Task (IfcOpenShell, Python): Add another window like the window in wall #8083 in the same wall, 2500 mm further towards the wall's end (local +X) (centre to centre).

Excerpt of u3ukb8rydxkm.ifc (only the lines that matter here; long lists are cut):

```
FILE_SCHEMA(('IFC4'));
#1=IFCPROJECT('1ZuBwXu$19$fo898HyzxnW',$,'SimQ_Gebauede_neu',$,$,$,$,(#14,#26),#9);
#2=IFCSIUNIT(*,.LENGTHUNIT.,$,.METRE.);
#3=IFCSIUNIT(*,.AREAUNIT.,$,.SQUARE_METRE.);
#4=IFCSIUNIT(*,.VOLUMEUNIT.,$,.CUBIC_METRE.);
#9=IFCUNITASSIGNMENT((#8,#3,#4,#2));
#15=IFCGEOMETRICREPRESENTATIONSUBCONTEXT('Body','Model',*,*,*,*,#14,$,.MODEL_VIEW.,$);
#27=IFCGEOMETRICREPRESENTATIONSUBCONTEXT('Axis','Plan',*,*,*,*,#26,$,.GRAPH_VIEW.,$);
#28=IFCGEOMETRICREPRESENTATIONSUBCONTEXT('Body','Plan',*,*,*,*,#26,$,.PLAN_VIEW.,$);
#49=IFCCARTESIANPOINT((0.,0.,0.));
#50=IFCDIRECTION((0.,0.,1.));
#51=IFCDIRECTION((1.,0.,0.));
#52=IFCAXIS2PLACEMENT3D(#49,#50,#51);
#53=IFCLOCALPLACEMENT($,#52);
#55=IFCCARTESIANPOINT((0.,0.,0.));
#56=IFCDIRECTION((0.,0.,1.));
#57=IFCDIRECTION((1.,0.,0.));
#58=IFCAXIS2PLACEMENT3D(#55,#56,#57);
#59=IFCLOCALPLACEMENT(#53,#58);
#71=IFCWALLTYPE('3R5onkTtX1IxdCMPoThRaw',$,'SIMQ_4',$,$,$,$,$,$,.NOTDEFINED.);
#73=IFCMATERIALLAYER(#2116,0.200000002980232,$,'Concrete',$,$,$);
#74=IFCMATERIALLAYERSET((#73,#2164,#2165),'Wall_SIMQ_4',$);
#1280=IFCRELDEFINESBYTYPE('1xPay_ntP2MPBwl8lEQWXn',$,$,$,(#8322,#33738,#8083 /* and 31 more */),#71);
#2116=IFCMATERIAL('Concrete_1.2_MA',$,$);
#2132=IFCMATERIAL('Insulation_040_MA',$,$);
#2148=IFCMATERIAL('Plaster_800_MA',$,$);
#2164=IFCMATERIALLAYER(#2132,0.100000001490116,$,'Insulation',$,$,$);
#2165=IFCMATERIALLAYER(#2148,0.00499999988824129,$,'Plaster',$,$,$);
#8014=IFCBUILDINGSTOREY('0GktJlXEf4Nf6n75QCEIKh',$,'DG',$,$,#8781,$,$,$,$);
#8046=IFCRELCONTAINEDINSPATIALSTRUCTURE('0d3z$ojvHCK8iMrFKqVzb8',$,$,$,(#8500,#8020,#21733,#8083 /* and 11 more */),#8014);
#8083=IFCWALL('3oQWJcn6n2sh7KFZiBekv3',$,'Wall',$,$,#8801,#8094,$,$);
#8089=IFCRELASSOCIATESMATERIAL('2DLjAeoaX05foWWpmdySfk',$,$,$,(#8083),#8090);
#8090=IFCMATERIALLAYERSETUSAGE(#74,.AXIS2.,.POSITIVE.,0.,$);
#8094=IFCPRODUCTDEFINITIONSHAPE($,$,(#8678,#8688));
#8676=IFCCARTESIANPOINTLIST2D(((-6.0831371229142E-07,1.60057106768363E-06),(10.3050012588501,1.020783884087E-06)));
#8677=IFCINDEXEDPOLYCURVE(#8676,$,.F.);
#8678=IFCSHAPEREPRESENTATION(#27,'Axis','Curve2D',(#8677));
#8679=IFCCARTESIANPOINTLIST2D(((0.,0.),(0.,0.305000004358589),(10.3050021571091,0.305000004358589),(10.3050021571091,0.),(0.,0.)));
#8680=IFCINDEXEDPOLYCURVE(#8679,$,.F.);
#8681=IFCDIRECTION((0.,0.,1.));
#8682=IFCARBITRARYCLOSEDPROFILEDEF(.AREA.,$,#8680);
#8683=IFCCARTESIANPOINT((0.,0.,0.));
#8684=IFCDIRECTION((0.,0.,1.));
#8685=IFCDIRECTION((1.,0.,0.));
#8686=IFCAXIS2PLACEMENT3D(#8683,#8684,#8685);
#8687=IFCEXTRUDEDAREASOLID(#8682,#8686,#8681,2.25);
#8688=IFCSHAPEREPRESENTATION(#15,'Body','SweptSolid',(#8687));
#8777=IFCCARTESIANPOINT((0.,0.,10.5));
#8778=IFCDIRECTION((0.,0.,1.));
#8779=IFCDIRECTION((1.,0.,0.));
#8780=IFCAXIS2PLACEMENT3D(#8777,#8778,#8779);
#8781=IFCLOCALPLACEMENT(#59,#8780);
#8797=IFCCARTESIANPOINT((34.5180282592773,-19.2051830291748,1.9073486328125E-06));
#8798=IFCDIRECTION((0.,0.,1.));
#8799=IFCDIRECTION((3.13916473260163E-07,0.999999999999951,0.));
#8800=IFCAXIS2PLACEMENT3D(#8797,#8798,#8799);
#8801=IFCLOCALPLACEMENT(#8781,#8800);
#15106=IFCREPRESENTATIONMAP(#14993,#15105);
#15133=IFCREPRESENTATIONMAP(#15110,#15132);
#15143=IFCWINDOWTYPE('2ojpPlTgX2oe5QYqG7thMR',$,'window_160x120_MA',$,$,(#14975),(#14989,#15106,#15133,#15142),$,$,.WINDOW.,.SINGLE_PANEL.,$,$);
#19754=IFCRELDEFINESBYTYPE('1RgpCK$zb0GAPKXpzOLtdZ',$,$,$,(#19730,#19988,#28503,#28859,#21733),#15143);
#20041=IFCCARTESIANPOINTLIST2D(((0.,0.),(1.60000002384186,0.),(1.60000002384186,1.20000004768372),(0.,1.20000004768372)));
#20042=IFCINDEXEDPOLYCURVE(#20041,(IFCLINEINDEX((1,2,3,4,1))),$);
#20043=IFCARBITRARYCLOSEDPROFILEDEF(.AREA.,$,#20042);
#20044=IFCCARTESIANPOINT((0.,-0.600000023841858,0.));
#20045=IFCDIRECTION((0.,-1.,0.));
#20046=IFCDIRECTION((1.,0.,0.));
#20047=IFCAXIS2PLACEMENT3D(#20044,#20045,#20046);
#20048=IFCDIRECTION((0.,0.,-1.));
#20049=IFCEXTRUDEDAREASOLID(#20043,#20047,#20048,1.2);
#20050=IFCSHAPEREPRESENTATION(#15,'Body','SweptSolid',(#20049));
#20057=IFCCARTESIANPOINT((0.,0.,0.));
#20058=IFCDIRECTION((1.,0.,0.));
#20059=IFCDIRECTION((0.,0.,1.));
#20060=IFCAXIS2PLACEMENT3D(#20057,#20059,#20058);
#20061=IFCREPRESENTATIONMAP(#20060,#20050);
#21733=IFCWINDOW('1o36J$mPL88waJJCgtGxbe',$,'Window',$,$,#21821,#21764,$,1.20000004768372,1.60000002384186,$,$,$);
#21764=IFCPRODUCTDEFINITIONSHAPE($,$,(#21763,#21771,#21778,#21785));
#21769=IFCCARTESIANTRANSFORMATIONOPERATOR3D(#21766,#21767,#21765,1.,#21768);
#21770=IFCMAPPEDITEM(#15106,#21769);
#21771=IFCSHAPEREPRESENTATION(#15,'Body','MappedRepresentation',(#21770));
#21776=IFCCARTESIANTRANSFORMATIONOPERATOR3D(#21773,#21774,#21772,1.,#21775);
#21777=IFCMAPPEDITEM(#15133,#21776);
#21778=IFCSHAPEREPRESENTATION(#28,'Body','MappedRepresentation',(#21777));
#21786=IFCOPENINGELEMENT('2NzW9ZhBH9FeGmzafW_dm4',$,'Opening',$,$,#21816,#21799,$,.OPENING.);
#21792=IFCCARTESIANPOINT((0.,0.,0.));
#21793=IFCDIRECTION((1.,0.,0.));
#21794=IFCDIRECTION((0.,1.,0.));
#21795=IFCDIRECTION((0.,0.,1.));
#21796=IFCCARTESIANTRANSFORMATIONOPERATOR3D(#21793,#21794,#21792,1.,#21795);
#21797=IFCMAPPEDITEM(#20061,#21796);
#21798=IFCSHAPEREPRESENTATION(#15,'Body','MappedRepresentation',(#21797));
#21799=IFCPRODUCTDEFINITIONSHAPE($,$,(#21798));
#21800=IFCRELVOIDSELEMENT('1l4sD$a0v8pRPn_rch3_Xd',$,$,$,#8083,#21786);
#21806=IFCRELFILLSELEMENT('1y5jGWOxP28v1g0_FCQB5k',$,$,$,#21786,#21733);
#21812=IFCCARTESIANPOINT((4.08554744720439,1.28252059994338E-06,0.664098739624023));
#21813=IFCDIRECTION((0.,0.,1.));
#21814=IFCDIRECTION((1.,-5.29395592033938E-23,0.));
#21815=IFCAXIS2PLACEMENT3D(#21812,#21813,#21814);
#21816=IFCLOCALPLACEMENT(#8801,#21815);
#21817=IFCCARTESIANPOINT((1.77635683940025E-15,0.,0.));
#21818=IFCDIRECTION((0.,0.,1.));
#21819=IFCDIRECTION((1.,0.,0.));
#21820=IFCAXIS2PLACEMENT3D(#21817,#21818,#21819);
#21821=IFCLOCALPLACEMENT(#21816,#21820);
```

```python
import ifcopenshell
import ifcopenshell.api.feature
import ifcopenshell.api.geometry
import ifcopenshell.api.root
import ifcopenshell.geom
import ifcopenshell.util.element
import ifcopenshell.util.placement
import ifcopenshell.util.shape

model = ifcopenshell.open("u3ukb8rydxkm.ifc")
settings = ifcopenshell.geom.settings()


def volume(element):
    """Net volume in cubic metres, openings subtracted."""
    shape = ifcopenshell.geom.create_shape(settings, element)
    return ifcopenshell.util.shape.get_volume(shape.geometry)


window = model.by_guid("1o36J$mPL88waJJCgtGxbe")
opening = window.FillsVoids[0].RelatingOpeningElement
wall = opening.VoidsElements[0].RelatingBuildingElement
before = volume(wall)
shift = ifcopenshell.util.placement.get_local_placement(wall.ObjectPlacement)[:3, 0] * 2.5

# copy_class copies the void relationship, type, container and properties, but no geometry.
new_opening = ifcopenshell.api.root.copy_class(model, product=opening)
new_opening.Representation = ifcopenshell.util.element.copy_deep(
    model, opening.Representation, exclude=["IfcGeometricRepresentationContext", "IfcRepresentationMap"]
)
new_window = ifcopenshell.api.root.copy_class(model, product=window)
new_window.Representation = ifcopenshell.util.element.copy_deep(
    model, window.Representation, exclude=["IfcGeometricRepresentationContext", "IfcRepresentationMap"]
)
ifcopenshell.api.feature.add_filling(model, opening=new_opening, element=new_window)

for old, new in ((opening, new_opening), (window, new_window)):
    matrix = ifcopenshell.util.placement.get_local_placement(old.ObjectPlacement)
    matrix[:3, 3] += shift
    ifcopenshell.api.geometry.edit_object_placement(model, product=new, matrix=matrix, is_si=False)

after = volume(wall)

print(f"wall volume {before:.3f} -> {after:.3f} m3")

model.write("u3ukb8rydxkm_v2.ifc")
```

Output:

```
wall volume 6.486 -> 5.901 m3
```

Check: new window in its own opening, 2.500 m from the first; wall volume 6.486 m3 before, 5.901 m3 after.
